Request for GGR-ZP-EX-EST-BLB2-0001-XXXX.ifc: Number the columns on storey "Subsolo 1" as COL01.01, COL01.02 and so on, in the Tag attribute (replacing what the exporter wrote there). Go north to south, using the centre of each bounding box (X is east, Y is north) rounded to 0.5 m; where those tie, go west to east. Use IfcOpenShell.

First a look at what the model holds.

```python
import ifcopenshell
import ifcopenshell.util.element
import ifcopenshell.util.placement

model = ifcopenshell.open("GGR-ZP-EX-EST-BLB2-0001-XXXX.ifc")
print(model.schema)
storey = next(s for s in model.by_type("IfcBuildingStorey") if s.Name == "Subsolo 1")
columns = [e for e in ifcopenshell.util.element.get_decomposition(storey) if e.is_a("IfcColumn")]
for e in sorted(columns, key=lambda e: e.id()):
    origin = ifcopenshell.util.placement.get_local_placement(e.ObjectPlacement)[:3, 3]
    print(e.id(), e.Tag, e.Name, origin.round(2) + 0.0, sep=" | ")
```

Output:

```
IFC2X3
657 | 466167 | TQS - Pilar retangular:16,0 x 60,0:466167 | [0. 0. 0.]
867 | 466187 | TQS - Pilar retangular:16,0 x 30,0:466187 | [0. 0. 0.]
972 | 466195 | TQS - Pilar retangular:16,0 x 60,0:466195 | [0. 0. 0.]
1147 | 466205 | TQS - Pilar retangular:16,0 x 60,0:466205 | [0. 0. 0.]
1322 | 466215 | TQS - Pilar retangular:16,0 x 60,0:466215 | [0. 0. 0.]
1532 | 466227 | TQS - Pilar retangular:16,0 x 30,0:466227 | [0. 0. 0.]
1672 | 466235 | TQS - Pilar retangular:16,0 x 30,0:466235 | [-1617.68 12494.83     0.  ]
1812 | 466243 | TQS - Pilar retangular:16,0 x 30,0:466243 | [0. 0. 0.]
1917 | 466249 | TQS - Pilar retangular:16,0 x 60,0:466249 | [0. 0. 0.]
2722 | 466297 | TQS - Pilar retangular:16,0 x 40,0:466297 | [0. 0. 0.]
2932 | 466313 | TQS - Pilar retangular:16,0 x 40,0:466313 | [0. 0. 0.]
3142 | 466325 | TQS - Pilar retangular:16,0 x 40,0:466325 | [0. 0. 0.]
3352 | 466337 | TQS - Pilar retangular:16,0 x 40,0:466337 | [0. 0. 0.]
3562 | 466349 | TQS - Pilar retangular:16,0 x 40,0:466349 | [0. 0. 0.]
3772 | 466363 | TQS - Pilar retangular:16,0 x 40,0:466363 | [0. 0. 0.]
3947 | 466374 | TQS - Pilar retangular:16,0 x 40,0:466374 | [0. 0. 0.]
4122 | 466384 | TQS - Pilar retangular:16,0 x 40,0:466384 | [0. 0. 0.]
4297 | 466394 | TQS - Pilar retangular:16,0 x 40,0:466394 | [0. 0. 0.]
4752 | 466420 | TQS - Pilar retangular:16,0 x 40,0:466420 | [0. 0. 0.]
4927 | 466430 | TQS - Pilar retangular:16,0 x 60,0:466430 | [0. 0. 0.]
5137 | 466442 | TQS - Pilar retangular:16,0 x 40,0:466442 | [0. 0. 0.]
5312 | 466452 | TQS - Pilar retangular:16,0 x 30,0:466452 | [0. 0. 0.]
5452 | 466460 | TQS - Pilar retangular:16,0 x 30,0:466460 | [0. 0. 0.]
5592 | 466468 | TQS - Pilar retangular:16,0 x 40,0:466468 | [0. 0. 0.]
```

```python
import ifcopenshell
import ifcopenshell.geom
import ifcopenshell.util.element
import ifcopenshell.util.shape

model = ifcopenshell.open("GGR-ZP-EX-EST-BLB2-0001-XXXX.ifc")
settings = ifcopenshell.geom.settings()
settings.set("use-world-coords", True)


def centre(element):
    shape = ifcopenshell.geom.create_shape(settings, element)
    return ifcopenshell.util.shape.get_bbox_centroid(shape.geometry)


storey = next(s for s in model.by_type("IfcBuildingStorey") if s.Name == "Subsolo 1")
columns = [e for e in ifcopenshell.util.element.get_decomposition(storey) if e.is_a("IfcColumn")]

# Insertion points can sit at a corner or the storey origin, so sort by the geometry (in metres).
centres = {e: centre(e) for e in columns}
columns.sort(key=lambda e: (-round(centres[e][1] / 0.5), centres[e][0]))

for i, e in enumerate(columns, start=1):
    number = f"COL01.{i:02d}"
    e.Tag = number
    print(e.id(), number)

model.write("GGR-ZP-EX-EST-BLB2-0001-XXXX_v2.ifc")
```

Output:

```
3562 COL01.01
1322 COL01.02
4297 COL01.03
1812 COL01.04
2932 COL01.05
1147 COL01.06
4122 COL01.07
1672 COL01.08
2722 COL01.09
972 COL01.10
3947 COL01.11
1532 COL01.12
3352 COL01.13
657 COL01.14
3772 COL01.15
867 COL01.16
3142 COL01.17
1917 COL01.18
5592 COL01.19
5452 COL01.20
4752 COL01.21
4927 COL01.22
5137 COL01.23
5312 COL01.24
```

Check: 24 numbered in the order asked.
